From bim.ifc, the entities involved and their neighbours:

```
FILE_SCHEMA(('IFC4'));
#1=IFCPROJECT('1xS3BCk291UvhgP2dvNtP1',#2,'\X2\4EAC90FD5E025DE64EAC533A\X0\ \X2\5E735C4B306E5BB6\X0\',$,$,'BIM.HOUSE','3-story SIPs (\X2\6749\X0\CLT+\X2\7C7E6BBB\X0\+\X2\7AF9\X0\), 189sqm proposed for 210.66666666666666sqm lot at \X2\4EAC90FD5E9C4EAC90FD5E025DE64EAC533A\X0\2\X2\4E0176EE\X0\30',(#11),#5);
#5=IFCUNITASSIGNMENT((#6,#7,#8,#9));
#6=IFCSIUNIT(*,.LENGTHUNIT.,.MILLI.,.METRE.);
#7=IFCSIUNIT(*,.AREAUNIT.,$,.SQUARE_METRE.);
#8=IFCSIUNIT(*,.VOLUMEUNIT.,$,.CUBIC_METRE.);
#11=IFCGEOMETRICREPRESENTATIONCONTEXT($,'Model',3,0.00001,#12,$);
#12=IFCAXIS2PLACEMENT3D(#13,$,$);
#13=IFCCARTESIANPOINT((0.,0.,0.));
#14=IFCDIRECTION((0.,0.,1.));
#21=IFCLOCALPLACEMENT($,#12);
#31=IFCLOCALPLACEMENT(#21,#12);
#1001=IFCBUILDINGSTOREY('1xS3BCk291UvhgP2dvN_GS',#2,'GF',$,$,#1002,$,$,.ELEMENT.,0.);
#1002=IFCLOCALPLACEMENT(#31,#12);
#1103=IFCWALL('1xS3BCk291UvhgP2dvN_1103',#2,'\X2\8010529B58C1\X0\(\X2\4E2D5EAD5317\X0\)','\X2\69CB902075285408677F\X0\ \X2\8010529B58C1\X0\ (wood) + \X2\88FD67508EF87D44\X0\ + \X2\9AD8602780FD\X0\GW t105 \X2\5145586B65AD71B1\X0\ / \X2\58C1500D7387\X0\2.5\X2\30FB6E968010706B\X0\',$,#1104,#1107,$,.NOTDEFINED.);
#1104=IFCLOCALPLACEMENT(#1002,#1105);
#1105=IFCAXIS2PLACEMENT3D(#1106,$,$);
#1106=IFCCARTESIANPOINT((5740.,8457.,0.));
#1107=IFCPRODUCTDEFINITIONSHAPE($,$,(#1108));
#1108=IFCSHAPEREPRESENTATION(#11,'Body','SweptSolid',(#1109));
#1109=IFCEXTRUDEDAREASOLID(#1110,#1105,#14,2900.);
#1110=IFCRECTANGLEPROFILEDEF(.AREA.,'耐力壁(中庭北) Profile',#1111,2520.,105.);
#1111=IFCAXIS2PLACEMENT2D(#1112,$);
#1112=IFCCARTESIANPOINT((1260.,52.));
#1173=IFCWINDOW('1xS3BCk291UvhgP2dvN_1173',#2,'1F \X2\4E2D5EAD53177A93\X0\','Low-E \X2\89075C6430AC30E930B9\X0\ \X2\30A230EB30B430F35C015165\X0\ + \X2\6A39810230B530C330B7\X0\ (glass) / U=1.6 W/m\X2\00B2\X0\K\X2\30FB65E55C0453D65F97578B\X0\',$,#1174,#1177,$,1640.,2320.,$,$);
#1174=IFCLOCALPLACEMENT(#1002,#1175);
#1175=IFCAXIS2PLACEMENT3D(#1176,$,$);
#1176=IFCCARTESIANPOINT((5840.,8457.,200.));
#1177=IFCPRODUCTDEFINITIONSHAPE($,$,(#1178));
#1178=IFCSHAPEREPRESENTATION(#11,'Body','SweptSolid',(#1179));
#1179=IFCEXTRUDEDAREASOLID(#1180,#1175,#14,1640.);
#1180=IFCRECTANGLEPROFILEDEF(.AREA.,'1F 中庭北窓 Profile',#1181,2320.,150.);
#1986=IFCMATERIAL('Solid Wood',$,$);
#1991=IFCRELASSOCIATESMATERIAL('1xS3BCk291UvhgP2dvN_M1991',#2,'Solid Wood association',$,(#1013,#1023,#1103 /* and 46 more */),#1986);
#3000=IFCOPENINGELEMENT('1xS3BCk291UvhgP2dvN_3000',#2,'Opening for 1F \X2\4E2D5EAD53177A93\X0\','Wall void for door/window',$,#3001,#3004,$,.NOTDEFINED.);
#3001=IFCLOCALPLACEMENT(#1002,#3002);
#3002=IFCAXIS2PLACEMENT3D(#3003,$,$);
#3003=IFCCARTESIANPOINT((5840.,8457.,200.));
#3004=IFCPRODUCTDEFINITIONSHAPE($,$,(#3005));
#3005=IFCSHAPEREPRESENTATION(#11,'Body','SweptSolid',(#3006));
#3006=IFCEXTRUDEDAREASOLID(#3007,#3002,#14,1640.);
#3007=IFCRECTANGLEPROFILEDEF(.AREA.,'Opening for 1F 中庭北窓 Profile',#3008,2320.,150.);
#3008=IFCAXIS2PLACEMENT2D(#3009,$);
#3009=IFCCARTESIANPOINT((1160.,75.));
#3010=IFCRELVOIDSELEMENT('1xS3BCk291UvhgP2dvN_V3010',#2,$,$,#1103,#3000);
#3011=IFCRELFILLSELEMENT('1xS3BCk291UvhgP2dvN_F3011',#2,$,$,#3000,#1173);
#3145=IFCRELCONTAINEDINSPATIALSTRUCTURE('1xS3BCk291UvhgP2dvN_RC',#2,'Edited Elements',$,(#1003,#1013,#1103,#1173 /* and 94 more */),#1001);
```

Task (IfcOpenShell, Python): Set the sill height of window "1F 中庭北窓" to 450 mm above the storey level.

```python
import numpy as np
import ifcopenshell
import ifcopenshell.api.geometry
import ifcopenshell.geom
import ifcopenshell.util.element
import ifcopenshell.util.placement
import ifcopenshell.util.shape
import ifcopenshell.util.unit

model = ifcopenshell.open("bim.ifc")
unit_scale = ifcopenshell.util.unit.calculate_unit_scale(model)

window = model.by_guid("1xS3BCk291UvhgP2dvN_1173")
opening = window.FillsVoids[0].RelatingOpeningElement
storey = ifcopenshell.util.element.get_container(window, ifc_class="IfcBuildingStorey")
level = ifcopenshell.util.placement.get_local_placement(storey.ObjectPlacement)[2, 3]

# The opening's origin need not be at the sill, so measure its lowest point.
shape = ifcopenshell.geom.create_shape(ifcopenshell.geom.settings(), opening)
bottom = ifcopenshell.util.shape.get_shape_bottom_elevation(shape, shape.geometry) / unit_scale
dz = level + 0.45 / unit_scale - bottom

shift = np.array([0.0, 0.0, dz])
# The window is not placed relative to its opening, so move both.
for product in (opening, window):
    matrix = ifcopenshell.util.placement.get_local_placement(product.ObjectPlacement)
    matrix[:3, 3] += shift
    ifcopenshell.api.geometry.edit_object_placement(model, product=product, matrix=matrix, is_si=False)

print(f"moved by {dz * unit_scale:+.3f} m")

model.write("bim_edited.ifc")
```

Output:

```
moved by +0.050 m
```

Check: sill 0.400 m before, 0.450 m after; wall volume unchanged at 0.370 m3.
